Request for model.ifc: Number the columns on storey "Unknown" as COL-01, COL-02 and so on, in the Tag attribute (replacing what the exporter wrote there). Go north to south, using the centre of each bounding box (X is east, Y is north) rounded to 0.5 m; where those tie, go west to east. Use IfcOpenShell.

First a look at what the model holds.

```python
import ifcopenshell
import ifcopenshell.util.element
import ifcopenshell.util.placement

model = ifcopenshell.open("model.ifc")
print(model.schema)
storey = next(s for s in model.by_type("IfcBuildingStorey") if s.Name == "Unknown")
columns = [e for e in ifcopenshell.util.element.get_decomposition(storey) if e.is_a("IfcColumn")]
for e in sorted(columns, key=lambda e: e.id()):
    origin = ifcopenshell.util.placement.get_local_placement(e.ObjectPlacement)[:3, 3]
    print(e.id(), e.Tag, e.Name, origin.round(2) + 0.0, sep=" | ")
```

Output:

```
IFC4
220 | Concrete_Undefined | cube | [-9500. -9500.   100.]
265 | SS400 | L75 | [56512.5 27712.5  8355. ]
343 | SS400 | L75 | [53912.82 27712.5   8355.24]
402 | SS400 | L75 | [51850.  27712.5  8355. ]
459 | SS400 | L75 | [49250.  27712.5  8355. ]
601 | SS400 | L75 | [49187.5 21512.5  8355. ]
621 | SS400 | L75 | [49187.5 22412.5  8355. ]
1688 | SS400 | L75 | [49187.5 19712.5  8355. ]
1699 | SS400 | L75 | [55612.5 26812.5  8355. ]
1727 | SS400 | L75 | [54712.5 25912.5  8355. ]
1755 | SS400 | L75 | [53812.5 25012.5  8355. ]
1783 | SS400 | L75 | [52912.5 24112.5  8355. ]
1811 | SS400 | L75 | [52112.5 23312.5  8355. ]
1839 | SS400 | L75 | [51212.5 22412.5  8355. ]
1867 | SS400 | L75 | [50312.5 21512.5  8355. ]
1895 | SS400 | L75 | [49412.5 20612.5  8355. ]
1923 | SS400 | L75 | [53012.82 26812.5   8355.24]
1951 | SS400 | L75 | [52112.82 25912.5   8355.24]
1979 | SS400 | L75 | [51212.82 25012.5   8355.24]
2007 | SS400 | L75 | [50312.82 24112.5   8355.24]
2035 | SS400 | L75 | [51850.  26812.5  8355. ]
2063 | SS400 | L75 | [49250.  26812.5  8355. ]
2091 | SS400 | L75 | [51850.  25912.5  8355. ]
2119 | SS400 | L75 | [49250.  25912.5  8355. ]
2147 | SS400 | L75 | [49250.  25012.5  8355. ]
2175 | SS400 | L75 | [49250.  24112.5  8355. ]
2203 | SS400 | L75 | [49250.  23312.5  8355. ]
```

```python
import ifcopenshell
import ifcopenshell.geom
import ifcopenshell.util.element
import ifcopenshell.util.shape

model = ifcopenshell.open("model.ifc")
settings = ifcopenshell.geom.settings()
settings.set("use-world-coords", True)


def centre(element):
    shape = ifcopenshell.geom.create_shape(settings, element)
    return ifcopenshell.util.shape.get_bbox_centroid(shape.geometry)


storey = next(s for s in model.by_type("IfcBuildingStorey") if s.Name == "Unknown")
columns = [e for e in ifcopenshell.util.element.get_decomposition(storey) if e.is_a("IfcColumn")]

# Insertion points can sit at a corner or the storey origin, so sort by the geometry (in metres).
centres = {e: centre(e) for e in columns}
columns.sort(key=lambda e: (-round(centres[e][1] / 0.5), centres[e][0]))

for i, e in enumerate(columns, start=1):
    number = f"COL-{i:02d}"
    e.Tag = number
    print(e.id(), number)

model.write("model_updated.ifc")
```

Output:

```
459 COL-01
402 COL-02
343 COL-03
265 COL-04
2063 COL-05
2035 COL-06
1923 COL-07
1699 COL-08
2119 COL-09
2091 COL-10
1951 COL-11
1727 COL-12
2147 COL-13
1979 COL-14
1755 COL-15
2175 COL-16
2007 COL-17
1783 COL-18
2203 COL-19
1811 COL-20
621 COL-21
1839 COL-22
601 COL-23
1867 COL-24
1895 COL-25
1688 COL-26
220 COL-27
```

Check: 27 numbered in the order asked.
